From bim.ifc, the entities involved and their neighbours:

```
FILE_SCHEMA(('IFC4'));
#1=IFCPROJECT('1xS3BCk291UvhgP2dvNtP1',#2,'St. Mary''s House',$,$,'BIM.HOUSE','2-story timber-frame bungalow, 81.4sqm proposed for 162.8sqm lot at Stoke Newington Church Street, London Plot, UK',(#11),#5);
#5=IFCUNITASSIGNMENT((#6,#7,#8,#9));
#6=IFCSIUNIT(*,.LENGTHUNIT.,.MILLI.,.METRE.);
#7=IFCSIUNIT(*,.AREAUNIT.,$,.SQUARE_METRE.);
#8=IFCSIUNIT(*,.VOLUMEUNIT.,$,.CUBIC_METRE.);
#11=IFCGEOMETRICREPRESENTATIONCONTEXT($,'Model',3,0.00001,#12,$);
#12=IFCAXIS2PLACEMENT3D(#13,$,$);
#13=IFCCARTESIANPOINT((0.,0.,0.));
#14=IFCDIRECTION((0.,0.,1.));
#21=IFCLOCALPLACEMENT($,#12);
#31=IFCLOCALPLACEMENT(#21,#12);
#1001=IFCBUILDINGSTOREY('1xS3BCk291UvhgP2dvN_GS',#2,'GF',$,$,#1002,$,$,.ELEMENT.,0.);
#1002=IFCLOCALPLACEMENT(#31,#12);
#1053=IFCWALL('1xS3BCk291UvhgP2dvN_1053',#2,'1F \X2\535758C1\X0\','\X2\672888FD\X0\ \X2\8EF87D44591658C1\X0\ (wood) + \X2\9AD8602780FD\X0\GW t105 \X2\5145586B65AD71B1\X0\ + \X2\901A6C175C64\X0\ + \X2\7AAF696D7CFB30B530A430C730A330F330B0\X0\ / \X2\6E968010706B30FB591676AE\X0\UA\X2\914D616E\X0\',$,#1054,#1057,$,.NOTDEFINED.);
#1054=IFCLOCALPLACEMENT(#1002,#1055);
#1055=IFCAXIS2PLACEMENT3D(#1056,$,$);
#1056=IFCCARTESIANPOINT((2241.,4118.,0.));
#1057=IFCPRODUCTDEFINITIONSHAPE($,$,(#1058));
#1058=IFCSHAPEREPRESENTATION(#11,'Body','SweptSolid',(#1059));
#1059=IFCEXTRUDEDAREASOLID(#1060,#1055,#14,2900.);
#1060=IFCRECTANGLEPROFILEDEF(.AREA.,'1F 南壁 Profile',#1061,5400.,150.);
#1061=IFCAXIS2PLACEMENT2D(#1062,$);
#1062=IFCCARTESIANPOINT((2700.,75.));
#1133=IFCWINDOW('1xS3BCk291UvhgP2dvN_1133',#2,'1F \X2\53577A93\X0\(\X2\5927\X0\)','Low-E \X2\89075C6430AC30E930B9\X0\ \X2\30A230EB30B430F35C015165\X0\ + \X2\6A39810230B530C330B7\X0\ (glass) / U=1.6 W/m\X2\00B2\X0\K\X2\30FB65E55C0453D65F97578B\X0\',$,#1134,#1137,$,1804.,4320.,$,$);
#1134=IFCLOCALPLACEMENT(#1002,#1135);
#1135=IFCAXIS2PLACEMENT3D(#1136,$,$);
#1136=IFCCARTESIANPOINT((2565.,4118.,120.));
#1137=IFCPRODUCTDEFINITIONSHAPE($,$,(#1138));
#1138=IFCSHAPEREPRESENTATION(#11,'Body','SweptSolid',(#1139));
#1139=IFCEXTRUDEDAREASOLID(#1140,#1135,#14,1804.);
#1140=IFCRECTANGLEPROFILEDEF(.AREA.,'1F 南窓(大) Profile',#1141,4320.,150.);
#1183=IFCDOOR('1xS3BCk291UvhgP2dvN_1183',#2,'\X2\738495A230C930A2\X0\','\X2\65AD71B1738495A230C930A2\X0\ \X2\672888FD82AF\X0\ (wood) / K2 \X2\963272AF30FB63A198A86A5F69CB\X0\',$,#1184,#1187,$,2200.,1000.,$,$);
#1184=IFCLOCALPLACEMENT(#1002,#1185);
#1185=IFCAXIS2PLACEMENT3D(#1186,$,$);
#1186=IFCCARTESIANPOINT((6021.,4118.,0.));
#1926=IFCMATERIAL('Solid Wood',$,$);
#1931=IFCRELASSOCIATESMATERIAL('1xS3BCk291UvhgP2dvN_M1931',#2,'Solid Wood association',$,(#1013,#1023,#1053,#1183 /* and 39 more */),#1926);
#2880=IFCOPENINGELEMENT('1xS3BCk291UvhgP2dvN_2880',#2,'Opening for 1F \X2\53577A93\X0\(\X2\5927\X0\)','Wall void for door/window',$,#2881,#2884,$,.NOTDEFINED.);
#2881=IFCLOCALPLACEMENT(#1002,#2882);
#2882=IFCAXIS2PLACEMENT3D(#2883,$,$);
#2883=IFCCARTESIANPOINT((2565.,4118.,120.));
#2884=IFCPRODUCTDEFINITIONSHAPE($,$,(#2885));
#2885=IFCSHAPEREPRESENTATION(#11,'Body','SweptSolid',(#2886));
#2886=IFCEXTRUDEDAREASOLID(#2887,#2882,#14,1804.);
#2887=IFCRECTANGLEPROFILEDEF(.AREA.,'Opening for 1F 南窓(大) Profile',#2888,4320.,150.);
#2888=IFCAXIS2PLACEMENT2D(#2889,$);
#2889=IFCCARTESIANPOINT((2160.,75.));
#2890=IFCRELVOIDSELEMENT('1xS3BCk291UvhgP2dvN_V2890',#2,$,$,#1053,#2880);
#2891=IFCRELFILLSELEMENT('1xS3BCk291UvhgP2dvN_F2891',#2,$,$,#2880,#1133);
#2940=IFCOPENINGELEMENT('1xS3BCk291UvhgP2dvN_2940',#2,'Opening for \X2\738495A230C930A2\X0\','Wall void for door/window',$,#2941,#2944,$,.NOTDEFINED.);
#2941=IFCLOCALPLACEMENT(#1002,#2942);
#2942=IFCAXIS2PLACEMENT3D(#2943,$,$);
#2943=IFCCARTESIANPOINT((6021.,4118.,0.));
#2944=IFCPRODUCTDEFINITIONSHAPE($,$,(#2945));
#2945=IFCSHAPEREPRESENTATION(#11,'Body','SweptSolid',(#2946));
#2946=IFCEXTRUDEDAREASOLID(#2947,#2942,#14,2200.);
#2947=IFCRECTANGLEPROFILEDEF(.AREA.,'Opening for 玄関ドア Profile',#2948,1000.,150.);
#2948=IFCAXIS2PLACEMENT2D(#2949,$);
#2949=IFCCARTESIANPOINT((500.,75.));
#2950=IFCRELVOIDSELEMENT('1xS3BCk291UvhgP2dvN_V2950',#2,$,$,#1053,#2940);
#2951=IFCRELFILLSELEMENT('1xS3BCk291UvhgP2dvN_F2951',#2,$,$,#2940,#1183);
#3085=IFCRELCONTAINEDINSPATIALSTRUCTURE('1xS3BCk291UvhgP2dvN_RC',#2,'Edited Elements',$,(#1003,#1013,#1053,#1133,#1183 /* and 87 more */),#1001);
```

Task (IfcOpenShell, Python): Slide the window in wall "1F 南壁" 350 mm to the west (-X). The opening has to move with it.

```python
import ifcopenshell
import ifcopenshell.api.geometry
import ifcopenshell.util.placement
import ifcopenshell.util.unit

model = ifcopenshell.open("bim.ifc")
unit_scale = ifcopenshell.util.unit.calculate_unit_scale(model)

window = model.by_guid("1xS3BCk291UvhgP2dvN_1133")
opening = window.FillsVoids[0].RelatingOpeningElement
wall = opening.VoidsElements[0].RelatingBuildingElement

wall_matrix = ifcopenshell.util.placement.get_local_placement(wall.ObjectPlacement)
shift = wall_matrix[:3, 0] * -0.35 / unit_scale
before = ifcopenshell.util.placement.get_local_placement(window.ObjectPlacement)[:3, 3].copy()

# The window is not placed relative to its opening, so move both.
for product in (opening, window):
    matrix = ifcopenshell.util.placement.get_local_placement(product.ObjectPlacement)
    matrix[:3, 3] += shift
    ifcopenshell.api.geometry.edit_object_placement(model, product=product, matrix=matrix, is_si=False)

after = ifcopenshell.util.placement.get_local_placement(window.ObjectPlacement)[:3, 3]
print("window moved by", (after - before).round(3) + 0.0)

model.write("bim_rev.ifc")
```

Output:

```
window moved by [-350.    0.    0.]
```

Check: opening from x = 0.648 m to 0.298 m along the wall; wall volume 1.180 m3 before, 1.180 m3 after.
